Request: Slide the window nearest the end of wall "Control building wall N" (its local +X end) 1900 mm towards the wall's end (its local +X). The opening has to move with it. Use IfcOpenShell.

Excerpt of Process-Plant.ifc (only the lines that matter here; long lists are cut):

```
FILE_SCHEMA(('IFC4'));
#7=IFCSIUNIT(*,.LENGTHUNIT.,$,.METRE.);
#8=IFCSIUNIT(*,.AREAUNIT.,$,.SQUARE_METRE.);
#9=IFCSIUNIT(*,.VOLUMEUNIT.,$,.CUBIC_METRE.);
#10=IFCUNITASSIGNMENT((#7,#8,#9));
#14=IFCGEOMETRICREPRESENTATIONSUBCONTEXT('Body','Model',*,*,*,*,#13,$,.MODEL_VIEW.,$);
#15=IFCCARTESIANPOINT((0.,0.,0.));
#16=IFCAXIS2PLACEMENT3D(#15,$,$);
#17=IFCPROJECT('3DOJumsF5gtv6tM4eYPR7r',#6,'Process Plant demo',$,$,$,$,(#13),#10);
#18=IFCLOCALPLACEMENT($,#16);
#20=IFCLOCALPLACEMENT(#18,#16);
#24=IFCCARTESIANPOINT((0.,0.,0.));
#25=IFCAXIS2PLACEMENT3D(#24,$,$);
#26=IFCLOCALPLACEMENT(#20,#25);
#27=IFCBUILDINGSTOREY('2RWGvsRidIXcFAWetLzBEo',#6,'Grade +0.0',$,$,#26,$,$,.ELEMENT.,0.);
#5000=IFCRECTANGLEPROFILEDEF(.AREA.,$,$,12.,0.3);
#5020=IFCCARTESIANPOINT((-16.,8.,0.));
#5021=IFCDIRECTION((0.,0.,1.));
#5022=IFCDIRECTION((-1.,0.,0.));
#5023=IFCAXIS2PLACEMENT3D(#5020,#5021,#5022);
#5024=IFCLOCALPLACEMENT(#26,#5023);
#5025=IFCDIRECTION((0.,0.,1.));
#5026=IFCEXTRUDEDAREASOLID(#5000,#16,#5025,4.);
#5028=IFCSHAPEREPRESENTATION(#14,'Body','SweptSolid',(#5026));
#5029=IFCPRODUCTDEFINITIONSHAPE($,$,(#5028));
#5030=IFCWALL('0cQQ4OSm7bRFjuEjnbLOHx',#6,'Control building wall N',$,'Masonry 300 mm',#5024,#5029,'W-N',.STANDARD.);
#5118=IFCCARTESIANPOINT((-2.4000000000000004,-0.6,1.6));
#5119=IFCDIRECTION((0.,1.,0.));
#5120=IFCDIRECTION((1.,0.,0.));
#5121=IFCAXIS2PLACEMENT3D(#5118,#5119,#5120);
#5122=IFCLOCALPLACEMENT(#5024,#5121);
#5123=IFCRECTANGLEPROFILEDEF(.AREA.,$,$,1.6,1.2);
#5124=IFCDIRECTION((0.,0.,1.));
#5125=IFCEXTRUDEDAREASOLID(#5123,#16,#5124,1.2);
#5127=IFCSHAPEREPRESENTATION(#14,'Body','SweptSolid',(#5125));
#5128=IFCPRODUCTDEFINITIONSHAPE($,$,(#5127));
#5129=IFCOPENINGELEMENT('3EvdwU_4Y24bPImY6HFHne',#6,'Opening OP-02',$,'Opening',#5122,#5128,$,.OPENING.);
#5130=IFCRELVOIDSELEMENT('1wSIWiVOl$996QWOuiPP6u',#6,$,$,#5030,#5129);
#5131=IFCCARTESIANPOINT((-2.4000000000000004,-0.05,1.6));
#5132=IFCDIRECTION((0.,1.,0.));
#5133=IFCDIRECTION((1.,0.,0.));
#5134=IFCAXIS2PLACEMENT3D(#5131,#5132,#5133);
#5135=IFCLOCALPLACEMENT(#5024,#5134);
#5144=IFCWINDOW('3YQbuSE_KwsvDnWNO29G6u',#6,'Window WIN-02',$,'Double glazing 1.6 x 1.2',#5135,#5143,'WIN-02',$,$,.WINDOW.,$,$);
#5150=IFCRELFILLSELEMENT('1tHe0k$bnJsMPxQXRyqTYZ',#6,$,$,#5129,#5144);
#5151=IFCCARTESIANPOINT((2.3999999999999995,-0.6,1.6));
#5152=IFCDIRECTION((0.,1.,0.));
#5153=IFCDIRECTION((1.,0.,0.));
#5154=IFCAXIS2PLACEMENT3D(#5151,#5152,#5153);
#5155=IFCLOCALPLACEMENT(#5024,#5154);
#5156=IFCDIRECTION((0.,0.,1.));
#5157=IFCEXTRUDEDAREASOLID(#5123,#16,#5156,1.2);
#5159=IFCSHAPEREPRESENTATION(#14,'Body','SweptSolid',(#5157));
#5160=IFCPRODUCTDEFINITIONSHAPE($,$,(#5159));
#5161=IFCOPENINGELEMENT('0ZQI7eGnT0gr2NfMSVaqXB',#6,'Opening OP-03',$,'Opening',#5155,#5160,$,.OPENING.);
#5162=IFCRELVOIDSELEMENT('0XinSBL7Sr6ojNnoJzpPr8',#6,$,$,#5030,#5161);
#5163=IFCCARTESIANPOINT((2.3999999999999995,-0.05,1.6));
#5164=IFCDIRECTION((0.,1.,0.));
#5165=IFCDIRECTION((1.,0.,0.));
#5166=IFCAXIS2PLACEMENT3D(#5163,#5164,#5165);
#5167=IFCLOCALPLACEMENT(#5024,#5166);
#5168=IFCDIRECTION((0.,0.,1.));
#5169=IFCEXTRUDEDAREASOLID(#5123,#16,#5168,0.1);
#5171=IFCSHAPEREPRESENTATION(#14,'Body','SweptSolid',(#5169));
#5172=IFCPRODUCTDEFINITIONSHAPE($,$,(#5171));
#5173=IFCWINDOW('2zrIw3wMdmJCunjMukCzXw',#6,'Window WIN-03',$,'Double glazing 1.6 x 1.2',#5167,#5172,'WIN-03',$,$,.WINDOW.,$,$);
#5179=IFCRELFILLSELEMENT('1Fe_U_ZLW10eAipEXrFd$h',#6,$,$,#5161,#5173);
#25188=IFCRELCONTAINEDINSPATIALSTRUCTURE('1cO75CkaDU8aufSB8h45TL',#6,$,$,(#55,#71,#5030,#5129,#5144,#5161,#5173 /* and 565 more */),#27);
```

```python
import ifcopenshell
import ifcopenshell.api.geometry
import ifcopenshell.util.placement
import ifcopenshell.util.unit

model = ifcopenshell.open("Process-Plant.ifc")
unit_scale = ifcopenshell.util.unit.calculate_unit_scale(model)

window = model.by_id(5173)
opening = window.FillsVoids[0].RelatingOpeningElement
wall = opening.VoidsElements[0].RelatingBuildingElement

wall_matrix = ifcopenshell.util.placement.get_local_placement(wall.ObjectPlacement)
shift = wall_matrix[:3, 0] * 1.9 / unit_scale
before = ifcopenshell.util.placement.get_local_placement(window.ObjectPlacement)[:3, 3].copy()

# The window is not placed relative to its opening, so move both.
for product in (opening, window):
    matrix = ifcopenshell.util.placement.get_local_placement(product.ObjectPlacement)
    matrix[:3, 3] += shift
    ifcopenshell.api.geometry.edit_object_placement(model, product=product, matrix=matrix, is_si=False)

after = ifcopenshell.util.placement.get_local_placement(window.ObjectPlacement)[:3, 3]
print("window moved by", (after - before).round(3) + 0.0)

model.write("Process-Plant-out.ifc")
```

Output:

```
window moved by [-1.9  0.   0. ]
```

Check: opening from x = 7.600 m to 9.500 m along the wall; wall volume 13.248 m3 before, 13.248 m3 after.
